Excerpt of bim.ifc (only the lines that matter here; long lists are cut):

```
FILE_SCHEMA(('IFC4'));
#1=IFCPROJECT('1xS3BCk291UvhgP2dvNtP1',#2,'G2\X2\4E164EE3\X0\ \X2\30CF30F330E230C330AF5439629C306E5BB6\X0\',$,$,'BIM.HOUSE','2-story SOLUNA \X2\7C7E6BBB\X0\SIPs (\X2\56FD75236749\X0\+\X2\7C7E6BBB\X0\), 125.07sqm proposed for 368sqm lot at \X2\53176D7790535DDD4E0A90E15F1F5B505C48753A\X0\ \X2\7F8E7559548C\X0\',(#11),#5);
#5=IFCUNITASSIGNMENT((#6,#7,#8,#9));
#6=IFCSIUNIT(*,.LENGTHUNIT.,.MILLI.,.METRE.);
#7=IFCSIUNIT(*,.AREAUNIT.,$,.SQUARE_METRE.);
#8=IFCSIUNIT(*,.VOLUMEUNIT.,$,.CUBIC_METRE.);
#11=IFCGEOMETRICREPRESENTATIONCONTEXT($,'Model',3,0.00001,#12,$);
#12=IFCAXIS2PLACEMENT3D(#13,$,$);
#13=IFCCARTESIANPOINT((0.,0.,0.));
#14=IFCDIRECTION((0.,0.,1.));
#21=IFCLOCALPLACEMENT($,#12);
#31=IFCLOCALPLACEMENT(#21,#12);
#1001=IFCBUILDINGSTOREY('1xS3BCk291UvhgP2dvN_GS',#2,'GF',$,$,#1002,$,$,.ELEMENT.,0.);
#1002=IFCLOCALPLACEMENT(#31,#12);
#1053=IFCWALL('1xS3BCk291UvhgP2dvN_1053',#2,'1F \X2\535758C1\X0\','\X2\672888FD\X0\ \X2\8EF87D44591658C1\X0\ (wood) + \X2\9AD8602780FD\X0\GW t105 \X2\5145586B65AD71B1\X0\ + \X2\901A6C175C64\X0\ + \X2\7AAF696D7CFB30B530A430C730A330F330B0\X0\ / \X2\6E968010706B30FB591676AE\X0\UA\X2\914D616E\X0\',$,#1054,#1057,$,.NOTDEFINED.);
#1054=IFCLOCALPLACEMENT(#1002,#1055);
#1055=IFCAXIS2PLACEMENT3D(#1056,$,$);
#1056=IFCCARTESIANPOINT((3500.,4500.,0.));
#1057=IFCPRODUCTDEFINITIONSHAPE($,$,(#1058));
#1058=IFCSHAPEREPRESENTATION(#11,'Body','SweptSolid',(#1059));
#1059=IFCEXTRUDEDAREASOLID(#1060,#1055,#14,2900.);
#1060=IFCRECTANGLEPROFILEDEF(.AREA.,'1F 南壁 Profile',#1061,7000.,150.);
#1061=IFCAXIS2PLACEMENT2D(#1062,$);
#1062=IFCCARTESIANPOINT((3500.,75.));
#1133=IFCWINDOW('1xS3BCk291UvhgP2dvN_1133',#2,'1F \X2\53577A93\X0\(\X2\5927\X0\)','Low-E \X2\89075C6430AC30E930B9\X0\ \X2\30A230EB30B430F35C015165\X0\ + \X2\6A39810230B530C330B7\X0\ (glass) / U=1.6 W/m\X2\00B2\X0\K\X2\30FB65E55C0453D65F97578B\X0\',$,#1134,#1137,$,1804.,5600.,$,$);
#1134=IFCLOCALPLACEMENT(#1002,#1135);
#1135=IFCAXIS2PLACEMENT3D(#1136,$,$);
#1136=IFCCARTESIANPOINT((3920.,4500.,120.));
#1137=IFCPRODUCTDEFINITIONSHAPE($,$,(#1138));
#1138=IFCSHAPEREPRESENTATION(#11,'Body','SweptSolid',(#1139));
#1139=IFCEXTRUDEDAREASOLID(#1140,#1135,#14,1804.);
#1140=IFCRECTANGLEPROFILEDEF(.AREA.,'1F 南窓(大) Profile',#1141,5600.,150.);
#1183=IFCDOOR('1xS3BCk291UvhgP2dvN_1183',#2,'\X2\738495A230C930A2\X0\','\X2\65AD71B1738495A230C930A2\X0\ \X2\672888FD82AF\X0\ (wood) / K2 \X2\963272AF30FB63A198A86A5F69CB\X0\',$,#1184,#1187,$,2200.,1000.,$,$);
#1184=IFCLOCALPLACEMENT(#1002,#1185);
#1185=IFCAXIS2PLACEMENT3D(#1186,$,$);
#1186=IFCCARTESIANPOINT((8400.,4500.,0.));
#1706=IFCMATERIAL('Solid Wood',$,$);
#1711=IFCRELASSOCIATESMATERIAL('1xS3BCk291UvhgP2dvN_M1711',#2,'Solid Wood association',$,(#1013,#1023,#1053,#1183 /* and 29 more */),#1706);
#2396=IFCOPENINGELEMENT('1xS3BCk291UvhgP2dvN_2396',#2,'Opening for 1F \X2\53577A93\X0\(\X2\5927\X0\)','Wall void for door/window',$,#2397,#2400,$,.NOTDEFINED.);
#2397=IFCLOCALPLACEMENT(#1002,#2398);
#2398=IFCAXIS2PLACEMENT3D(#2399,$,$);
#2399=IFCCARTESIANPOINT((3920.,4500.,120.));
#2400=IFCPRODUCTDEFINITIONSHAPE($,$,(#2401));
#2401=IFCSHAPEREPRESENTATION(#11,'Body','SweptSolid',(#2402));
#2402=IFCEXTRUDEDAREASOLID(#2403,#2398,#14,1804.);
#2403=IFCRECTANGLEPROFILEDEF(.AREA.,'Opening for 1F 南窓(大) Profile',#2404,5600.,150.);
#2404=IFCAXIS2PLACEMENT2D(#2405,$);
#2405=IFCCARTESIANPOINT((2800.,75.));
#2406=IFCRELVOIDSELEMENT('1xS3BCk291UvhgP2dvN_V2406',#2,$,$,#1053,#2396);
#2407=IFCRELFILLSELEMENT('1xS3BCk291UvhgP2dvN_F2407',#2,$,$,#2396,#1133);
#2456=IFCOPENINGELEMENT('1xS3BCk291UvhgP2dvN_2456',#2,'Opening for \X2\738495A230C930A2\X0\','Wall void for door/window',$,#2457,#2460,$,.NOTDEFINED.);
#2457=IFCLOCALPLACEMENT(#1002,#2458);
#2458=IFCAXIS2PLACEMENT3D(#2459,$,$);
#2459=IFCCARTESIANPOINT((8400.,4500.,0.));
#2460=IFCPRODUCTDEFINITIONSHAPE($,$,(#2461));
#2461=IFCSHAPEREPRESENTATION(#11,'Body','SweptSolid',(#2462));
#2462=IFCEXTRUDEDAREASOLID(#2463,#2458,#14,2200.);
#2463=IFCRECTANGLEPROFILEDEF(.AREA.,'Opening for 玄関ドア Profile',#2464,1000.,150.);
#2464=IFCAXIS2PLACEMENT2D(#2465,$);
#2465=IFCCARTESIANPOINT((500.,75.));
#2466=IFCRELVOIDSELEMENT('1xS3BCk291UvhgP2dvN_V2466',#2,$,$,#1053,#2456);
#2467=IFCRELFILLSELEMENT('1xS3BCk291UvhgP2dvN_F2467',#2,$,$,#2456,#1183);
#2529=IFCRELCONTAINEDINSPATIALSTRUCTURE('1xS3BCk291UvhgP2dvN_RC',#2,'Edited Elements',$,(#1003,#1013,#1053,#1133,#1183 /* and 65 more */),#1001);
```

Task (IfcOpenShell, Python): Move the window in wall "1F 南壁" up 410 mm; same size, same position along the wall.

```python
import numpy as np
import ifcopenshell
import ifcopenshell.api.geometry
import ifcopenshell.util.placement
import ifcopenshell.util.unit

model = ifcopenshell.open("bim.ifc")
unit_scale = ifcopenshell.util.unit.calculate_unit_scale(model)

window = model.by_id(1133)
opening = window.FillsVoids[0].RelatingOpeningElement
dz = 410.0

shift = np.array([0.0, 0.0, dz])
# The window is not placed relative to its opening, so move both.
for product in (opening, window):
    matrix = ifcopenshell.util.placement.get_local_placement(product.ObjectPlacement)
    matrix[:3, 3] += shift
    ifcopenshell.api.geometry.edit_object_placement(model, product=product, matrix=matrix, is_si=False)

print(f"moved by {dz * unit_scale:+.3f} m")

model.write("bim-out.ifc")
```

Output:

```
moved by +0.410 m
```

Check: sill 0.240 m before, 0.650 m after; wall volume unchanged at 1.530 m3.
